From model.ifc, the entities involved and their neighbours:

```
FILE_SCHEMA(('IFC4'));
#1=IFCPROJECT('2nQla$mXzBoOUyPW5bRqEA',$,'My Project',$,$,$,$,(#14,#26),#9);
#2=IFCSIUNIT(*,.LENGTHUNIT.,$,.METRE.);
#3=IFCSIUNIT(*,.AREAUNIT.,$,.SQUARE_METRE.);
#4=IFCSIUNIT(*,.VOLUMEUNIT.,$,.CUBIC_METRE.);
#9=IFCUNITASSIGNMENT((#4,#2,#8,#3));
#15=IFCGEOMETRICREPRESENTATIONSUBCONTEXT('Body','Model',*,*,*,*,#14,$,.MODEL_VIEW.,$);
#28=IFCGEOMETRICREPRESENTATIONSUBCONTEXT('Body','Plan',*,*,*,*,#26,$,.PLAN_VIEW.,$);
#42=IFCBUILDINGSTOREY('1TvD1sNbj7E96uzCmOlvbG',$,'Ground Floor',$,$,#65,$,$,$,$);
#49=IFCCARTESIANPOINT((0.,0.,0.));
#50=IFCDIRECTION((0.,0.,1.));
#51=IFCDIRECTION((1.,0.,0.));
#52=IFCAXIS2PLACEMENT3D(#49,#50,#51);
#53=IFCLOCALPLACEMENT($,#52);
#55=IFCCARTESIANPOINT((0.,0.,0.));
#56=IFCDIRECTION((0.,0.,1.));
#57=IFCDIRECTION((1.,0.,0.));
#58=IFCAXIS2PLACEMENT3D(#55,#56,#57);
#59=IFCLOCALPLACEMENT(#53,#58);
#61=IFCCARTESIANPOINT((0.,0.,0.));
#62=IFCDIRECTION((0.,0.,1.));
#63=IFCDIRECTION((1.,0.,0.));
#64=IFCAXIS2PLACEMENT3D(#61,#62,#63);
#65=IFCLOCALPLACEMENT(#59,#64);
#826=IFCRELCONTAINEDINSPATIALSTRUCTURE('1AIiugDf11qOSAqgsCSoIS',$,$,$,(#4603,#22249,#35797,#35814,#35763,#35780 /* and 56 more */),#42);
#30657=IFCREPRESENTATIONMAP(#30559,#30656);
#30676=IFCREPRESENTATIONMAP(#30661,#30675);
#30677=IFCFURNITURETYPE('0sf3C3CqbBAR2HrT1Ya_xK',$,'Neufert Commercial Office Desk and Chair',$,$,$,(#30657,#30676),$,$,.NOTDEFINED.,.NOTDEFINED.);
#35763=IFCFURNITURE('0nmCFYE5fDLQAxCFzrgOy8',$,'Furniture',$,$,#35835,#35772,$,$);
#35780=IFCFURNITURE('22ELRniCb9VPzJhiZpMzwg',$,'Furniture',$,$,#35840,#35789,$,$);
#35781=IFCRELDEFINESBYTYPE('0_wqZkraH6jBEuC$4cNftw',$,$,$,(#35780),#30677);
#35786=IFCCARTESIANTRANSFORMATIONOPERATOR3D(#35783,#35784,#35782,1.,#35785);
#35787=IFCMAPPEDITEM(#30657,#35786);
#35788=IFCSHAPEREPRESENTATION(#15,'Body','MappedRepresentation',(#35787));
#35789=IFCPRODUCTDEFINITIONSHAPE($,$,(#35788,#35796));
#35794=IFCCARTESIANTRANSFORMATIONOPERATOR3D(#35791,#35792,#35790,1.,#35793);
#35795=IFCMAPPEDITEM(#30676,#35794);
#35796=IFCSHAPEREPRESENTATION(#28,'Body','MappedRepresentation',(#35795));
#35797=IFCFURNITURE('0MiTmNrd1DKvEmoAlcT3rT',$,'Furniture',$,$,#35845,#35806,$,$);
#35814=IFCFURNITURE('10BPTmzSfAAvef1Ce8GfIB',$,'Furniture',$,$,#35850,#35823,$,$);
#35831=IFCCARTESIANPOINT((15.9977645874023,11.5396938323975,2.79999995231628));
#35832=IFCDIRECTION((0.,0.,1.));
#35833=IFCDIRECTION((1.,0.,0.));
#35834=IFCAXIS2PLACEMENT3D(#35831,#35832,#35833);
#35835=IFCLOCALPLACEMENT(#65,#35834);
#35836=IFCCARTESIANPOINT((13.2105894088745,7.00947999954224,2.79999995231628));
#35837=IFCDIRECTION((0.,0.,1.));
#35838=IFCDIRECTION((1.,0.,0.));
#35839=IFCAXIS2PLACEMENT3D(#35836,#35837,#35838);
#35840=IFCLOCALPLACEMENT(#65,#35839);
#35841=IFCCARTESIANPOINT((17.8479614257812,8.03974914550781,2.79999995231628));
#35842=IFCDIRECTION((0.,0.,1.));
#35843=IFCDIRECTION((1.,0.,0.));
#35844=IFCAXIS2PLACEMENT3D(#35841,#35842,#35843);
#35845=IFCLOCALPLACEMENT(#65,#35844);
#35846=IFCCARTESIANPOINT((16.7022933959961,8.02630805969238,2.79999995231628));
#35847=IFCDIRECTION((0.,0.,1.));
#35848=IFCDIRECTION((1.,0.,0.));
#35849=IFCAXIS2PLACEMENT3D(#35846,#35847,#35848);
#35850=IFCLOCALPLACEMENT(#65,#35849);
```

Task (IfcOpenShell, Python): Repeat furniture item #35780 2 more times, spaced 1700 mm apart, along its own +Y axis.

```python
import ifcopenshell
import ifcopenshell.api.geometry
import ifcopenshell.api.root
import ifcopenshell.util.element
import ifcopenshell.util.placement
import ifcopenshell.util.unit

model = ifcopenshell.open("model.ifc")
unit_scale = ifcopenshell.util.unit.calculate_unit_scale(model)

source = model.by_guid("22ELRniCb9VPzJhiZpMzwg")
base = ifcopenshell.util.placement.get_local_placement(source.ObjectPlacement)
step = base[:3, 1] * 1.7 / unit_scale

for i in range(1, 3):
    copy = ifcopenshell.api.root.copy_class(model, product=source)
    copy.Representation = ifcopenshell.util.element.copy_deep(
        model, source.Representation, exclude=["IfcGeometricRepresentationContext", "IfcRepresentationMap"]
    )
    matrix = base.copy()
    matrix[:3, 3] += i * step
    print("added at", matrix[:3, 3].round(3) + 0.0)
    ifcopenshell.api.geometry.edit_object_placement(model, product=copy, matrix=matrix, is_si=False)

model.write("model_rev.ifc")
```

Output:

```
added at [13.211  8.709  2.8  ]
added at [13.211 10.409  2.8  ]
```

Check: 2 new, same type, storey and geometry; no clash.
